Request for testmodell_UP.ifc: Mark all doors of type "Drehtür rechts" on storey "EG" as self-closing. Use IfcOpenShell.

First a look at what the model holds.

```python
import ifcopenshell
import ifcopenshell.util.element

model = ifcopenshell.open("testmodell_UP.ifc")
print(model.schema)
storey = next(s for s in model.by_type("IfcBuildingStorey") if s.Name == "EG")
doors = [e for e in ifcopenshell.util.element.get_decomposition(storey) if e.is_a("IfcDoor")]
seen = {}
for e in doors:
    element_type = ifcopenshell.util.element.get_type(e)
    key = (element_type.Name if element_type != e and element_type else None, ifcopenshell.util.element.get_pset(e, "Pset_DoorCommon", "SelfClosing"))
    seen[key] = seen.get(key, 0) + 1
for (name, value), count in sorted(seen.items(), key=str):
    print(count, "x", name, "|", value)
```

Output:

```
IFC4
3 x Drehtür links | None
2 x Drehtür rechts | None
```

```python
import ifcopenshell
import ifcopenshell.api.pset
import ifcopenshell.util.element

model = ifcopenshell.open("testmodell_UP.ifc")

storey = next(s for s in model.by_type("IfcBuildingStorey") if s.Name == "EG")
doors = [e for e in ifcopenshell.util.element.get_decomposition(storey) if e.is_a("IfcDoor")]

count = 0
for e in doors:
    element_type = ifcopenshell.util.element.get_type(e)
    if element_type in (None, e) or element_type.Name != "Drehtür rechts":
        continue
    # add_pset returns the element's existing set when there is one.
    pset = ifcopenshell.api.pset.add_pset(model, product=e, name="Pset_DoorCommon")
    ifcopenshell.api.pset.edit_pset(model, pset=pset, properties={"SelfClosing": True})
    count += 1

print(count, "doors updated")

model.write("testmodell_UP_rev.ifc")
```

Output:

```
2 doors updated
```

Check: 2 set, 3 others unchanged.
